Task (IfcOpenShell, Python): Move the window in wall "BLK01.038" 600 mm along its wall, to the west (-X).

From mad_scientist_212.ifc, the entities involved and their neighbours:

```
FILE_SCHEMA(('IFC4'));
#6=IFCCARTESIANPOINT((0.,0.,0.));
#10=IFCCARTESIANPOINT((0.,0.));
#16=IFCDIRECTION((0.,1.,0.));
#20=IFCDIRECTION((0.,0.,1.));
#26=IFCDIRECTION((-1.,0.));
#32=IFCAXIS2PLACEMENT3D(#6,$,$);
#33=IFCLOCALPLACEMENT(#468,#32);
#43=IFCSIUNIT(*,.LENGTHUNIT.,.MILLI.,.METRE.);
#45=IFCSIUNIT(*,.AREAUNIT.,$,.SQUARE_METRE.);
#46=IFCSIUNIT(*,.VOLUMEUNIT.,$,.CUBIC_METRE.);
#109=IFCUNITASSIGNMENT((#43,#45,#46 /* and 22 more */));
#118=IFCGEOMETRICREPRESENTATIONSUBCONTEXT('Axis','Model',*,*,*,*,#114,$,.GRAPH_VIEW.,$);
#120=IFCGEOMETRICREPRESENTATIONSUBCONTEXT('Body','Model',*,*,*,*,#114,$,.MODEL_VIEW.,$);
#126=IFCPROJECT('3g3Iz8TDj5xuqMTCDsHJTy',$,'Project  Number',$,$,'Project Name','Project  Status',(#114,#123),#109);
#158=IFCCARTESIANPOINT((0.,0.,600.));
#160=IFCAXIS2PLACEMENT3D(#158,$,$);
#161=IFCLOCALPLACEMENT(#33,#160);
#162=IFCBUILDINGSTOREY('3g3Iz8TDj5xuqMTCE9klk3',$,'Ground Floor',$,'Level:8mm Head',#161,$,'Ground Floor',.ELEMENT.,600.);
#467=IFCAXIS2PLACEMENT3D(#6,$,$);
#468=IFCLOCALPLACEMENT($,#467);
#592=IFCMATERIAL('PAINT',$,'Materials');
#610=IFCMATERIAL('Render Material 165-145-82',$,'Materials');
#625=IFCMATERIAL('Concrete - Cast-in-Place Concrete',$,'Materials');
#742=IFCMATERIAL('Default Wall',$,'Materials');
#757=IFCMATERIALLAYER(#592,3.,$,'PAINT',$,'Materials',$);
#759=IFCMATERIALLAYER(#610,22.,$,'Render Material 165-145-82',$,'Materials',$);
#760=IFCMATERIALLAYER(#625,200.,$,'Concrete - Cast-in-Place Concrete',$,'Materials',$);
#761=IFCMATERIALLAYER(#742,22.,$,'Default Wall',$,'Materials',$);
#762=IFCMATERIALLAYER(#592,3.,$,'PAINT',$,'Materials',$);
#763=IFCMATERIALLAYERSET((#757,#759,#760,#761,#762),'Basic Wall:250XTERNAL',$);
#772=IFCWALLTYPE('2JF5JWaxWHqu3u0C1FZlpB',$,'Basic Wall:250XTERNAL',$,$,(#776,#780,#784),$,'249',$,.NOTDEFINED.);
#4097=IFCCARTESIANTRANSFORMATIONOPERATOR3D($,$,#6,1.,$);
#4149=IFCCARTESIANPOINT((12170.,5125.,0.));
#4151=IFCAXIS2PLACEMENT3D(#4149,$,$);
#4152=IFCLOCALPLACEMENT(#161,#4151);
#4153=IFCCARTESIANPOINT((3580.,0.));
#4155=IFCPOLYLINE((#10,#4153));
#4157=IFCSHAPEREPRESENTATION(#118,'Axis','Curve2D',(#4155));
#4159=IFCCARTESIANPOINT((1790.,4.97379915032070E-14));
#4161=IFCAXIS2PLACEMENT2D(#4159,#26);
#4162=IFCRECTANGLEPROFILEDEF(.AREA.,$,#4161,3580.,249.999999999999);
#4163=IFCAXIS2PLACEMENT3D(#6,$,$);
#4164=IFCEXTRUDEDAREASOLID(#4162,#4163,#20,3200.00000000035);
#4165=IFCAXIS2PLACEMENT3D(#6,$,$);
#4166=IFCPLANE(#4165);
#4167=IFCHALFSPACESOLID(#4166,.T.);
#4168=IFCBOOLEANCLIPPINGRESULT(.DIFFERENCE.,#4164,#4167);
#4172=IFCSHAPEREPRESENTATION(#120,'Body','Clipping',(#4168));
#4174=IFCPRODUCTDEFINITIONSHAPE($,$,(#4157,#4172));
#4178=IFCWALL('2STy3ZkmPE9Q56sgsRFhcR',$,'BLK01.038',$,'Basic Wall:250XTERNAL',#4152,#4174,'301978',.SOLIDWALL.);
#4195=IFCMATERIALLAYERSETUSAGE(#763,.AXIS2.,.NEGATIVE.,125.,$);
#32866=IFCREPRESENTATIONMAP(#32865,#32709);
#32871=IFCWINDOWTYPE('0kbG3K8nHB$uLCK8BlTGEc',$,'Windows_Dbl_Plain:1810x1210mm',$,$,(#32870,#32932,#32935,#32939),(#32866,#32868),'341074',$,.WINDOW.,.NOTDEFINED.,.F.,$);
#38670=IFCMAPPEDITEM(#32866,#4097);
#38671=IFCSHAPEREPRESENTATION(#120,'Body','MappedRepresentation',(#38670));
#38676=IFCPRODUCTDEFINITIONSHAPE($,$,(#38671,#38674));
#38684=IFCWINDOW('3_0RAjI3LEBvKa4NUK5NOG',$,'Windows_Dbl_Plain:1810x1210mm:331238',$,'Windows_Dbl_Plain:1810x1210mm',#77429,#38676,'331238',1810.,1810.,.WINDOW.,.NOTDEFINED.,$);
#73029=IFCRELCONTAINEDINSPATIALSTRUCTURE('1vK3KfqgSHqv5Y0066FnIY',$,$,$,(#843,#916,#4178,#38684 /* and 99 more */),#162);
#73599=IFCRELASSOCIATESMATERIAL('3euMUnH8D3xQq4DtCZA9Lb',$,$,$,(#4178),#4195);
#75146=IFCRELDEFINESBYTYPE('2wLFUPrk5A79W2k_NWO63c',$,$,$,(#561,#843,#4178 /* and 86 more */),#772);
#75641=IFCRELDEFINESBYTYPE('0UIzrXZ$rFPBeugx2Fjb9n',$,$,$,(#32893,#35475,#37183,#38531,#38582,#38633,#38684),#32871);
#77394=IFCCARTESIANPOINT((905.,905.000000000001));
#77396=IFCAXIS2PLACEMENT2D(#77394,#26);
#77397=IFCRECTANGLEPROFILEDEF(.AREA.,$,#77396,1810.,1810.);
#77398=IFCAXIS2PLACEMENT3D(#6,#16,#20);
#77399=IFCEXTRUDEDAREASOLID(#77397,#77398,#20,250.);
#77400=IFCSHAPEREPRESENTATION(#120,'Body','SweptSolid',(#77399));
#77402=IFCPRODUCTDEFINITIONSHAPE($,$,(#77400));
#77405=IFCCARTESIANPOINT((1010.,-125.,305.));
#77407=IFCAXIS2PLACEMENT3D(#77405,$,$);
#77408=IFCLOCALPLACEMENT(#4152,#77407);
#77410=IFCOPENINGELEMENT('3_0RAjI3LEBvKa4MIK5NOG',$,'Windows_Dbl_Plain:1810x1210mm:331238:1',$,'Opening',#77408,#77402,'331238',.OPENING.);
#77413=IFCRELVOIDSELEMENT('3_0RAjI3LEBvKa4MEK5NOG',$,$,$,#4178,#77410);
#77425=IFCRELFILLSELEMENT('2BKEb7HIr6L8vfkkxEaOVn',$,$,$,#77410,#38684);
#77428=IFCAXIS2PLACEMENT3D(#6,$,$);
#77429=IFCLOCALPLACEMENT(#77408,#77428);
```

```python
import ifcopenshell
import ifcopenshell.api.geometry
import ifcopenshell.util.placement
import ifcopenshell.util.unit

model = ifcopenshell.open("mad_scientist_212.ifc")
unit_scale = ifcopenshell.util.unit.calculate_unit_scale(model)

window = model.by_id(38684)
opening = window.FillsVoids[0].RelatingOpeningElement
wall = opening.VoidsElements[0].RelatingBuildingElement

wall_matrix = ifcopenshell.util.placement.get_local_placement(wall.ObjectPlacement)
shift = wall_matrix[:3, 0] * -0.6 / unit_scale
before = ifcopenshell.util.placement.get_local_placement(window.ObjectPlacement)[:3, 3].copy()

# The window is placed relative to its opening, so it follows when the opening moves.
matrix = ifcopenshell.util.placement.get_local_placement(opening.ObjectPlacement)
matrix[:3, 3] += shift
ifcopenshell.api.geometry.edit_object_placement(
    model, product=opening, matrix=matrix, is_si=False, should_transform_children=True
)

after = ifcopenshell.util.placement.get_local_placement(window.ObjectPlacement)[:3, 3]
print("window moved by", (after - before).round(3) + 0.0)

model.write("mad_scientist_212_edited.ifc")
```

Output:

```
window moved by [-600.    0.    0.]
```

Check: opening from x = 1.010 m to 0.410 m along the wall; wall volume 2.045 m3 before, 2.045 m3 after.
